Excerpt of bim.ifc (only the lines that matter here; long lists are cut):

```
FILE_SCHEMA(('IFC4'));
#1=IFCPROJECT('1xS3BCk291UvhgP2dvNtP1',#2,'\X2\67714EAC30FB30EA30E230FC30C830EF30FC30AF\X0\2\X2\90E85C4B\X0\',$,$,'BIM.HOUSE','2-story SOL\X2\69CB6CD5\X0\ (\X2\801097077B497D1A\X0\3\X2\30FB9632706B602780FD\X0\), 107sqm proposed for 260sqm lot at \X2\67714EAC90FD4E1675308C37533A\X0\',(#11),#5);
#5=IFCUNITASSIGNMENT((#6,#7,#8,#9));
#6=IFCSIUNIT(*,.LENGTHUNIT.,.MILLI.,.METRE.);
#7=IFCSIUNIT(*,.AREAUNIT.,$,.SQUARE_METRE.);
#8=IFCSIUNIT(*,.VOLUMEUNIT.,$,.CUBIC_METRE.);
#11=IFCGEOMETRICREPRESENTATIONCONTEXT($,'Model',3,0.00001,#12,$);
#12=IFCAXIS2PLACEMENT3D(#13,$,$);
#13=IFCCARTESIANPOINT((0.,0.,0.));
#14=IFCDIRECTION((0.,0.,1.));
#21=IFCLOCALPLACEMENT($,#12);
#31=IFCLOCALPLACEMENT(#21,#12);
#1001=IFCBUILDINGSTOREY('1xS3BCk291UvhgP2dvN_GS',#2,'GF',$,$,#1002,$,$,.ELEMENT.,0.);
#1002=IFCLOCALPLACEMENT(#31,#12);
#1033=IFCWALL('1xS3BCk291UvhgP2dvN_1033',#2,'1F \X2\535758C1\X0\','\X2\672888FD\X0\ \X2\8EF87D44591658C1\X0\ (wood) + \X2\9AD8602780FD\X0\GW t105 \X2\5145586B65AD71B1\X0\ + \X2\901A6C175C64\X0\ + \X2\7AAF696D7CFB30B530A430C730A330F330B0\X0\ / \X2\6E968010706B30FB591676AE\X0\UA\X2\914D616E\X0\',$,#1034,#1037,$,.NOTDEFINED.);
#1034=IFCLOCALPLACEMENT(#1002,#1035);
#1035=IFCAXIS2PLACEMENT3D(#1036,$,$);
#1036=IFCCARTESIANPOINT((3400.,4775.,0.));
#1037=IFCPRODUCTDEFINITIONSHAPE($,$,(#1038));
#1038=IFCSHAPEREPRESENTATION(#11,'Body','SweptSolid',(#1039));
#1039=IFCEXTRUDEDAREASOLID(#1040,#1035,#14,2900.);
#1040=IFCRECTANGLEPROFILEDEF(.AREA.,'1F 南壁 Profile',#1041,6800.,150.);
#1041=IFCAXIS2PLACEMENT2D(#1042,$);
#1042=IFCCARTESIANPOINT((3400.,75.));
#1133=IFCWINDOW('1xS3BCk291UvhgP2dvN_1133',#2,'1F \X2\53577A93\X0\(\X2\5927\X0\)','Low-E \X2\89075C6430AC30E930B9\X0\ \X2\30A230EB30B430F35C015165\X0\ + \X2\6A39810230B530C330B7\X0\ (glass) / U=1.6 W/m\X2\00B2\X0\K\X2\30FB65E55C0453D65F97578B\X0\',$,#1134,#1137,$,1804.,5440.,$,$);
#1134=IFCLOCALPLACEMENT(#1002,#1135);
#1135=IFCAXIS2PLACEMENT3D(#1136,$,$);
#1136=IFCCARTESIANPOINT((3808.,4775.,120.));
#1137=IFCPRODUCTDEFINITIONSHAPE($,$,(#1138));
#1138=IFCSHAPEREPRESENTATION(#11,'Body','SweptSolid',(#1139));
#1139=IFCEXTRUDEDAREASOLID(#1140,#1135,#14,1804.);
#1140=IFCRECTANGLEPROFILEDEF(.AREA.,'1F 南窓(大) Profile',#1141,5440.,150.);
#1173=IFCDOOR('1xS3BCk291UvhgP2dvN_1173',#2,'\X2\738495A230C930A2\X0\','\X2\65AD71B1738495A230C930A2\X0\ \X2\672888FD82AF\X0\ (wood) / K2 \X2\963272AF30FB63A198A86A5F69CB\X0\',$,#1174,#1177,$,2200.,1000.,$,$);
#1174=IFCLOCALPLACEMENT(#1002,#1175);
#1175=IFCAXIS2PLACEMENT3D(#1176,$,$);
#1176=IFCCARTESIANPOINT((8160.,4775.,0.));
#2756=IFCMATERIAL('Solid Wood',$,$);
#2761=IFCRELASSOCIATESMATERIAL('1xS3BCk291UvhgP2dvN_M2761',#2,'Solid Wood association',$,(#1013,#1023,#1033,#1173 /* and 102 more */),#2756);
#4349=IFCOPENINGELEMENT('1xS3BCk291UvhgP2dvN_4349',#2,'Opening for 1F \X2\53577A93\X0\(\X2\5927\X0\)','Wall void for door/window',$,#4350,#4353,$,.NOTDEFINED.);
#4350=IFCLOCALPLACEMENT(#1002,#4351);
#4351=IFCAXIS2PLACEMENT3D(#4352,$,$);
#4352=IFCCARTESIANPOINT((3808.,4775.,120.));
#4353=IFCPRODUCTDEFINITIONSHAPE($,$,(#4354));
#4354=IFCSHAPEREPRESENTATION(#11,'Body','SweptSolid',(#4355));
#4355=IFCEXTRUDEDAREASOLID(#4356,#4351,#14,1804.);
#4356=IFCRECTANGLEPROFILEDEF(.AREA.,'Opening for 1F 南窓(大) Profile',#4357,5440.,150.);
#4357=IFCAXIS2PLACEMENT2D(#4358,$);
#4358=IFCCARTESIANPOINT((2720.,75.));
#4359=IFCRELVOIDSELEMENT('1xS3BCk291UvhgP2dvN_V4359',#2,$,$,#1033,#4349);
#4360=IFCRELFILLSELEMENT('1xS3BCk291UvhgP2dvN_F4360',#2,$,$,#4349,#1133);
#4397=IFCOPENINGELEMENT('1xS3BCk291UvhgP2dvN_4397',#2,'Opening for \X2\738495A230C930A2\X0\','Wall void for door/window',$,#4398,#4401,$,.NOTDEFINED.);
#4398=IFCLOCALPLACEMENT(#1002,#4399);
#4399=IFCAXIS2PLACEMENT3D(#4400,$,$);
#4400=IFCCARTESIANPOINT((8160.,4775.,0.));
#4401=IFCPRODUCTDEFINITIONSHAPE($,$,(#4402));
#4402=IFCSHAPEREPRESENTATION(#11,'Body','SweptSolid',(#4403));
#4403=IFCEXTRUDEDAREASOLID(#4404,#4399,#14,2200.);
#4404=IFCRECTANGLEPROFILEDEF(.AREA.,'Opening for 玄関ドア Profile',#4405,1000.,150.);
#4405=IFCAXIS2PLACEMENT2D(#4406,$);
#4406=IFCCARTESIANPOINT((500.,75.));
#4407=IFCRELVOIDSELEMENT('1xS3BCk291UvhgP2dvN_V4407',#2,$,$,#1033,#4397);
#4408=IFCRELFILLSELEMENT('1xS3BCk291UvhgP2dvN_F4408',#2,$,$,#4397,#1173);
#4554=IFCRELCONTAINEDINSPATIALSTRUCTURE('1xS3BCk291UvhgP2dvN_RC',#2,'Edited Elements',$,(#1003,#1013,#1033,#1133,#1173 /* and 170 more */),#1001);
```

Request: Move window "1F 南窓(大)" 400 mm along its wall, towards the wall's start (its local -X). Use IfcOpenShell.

```python
import ifcopenshell
import ifcopenshell.api.geometry
import ifcopenshell.util.placement
import ifcopenshell.util.unit

model = ifcopenshell.open("bim.ifc")
unit_scale = ifcopenshell.util.unit.calculate_unit_scale(model)

window = model.by_id(1133)
opening = window.FillsVoids[0].RelatingOpeningElement
wall = opening.VoidsElements[0].RelatingBuildingElement

wall_matrix = ifcopenshell.util.placement.get_local_placement(wall.ObjectPlacement)
shift = wall_matrix[:3, 0] * -0.4 / unit_scale
before = ifcopenshell.util.placement.get_local_placement(window.ObjectPlacement)[:3, 3].copy()

# The window is not placed relative to its opening, so move both.
for product in (opening, window):
    matrix = ifcopenshell.util.placement.get_local_placement(product.ObjectPlacement)
    matrix[:3, 3] += shift
    ifcopenshell.api.geometry.edit_object_placement(model, product=product, matrix=matrix, is_si=False)

after = ifcopenshell.util.placement.get_local_placement(window.ObjectPlacement)[:3, 3]
print("window moved by", (after - before).round(3) + 0.0)

model.write("bim_v2.ifc")
```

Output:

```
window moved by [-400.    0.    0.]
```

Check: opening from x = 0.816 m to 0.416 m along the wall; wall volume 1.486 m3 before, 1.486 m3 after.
